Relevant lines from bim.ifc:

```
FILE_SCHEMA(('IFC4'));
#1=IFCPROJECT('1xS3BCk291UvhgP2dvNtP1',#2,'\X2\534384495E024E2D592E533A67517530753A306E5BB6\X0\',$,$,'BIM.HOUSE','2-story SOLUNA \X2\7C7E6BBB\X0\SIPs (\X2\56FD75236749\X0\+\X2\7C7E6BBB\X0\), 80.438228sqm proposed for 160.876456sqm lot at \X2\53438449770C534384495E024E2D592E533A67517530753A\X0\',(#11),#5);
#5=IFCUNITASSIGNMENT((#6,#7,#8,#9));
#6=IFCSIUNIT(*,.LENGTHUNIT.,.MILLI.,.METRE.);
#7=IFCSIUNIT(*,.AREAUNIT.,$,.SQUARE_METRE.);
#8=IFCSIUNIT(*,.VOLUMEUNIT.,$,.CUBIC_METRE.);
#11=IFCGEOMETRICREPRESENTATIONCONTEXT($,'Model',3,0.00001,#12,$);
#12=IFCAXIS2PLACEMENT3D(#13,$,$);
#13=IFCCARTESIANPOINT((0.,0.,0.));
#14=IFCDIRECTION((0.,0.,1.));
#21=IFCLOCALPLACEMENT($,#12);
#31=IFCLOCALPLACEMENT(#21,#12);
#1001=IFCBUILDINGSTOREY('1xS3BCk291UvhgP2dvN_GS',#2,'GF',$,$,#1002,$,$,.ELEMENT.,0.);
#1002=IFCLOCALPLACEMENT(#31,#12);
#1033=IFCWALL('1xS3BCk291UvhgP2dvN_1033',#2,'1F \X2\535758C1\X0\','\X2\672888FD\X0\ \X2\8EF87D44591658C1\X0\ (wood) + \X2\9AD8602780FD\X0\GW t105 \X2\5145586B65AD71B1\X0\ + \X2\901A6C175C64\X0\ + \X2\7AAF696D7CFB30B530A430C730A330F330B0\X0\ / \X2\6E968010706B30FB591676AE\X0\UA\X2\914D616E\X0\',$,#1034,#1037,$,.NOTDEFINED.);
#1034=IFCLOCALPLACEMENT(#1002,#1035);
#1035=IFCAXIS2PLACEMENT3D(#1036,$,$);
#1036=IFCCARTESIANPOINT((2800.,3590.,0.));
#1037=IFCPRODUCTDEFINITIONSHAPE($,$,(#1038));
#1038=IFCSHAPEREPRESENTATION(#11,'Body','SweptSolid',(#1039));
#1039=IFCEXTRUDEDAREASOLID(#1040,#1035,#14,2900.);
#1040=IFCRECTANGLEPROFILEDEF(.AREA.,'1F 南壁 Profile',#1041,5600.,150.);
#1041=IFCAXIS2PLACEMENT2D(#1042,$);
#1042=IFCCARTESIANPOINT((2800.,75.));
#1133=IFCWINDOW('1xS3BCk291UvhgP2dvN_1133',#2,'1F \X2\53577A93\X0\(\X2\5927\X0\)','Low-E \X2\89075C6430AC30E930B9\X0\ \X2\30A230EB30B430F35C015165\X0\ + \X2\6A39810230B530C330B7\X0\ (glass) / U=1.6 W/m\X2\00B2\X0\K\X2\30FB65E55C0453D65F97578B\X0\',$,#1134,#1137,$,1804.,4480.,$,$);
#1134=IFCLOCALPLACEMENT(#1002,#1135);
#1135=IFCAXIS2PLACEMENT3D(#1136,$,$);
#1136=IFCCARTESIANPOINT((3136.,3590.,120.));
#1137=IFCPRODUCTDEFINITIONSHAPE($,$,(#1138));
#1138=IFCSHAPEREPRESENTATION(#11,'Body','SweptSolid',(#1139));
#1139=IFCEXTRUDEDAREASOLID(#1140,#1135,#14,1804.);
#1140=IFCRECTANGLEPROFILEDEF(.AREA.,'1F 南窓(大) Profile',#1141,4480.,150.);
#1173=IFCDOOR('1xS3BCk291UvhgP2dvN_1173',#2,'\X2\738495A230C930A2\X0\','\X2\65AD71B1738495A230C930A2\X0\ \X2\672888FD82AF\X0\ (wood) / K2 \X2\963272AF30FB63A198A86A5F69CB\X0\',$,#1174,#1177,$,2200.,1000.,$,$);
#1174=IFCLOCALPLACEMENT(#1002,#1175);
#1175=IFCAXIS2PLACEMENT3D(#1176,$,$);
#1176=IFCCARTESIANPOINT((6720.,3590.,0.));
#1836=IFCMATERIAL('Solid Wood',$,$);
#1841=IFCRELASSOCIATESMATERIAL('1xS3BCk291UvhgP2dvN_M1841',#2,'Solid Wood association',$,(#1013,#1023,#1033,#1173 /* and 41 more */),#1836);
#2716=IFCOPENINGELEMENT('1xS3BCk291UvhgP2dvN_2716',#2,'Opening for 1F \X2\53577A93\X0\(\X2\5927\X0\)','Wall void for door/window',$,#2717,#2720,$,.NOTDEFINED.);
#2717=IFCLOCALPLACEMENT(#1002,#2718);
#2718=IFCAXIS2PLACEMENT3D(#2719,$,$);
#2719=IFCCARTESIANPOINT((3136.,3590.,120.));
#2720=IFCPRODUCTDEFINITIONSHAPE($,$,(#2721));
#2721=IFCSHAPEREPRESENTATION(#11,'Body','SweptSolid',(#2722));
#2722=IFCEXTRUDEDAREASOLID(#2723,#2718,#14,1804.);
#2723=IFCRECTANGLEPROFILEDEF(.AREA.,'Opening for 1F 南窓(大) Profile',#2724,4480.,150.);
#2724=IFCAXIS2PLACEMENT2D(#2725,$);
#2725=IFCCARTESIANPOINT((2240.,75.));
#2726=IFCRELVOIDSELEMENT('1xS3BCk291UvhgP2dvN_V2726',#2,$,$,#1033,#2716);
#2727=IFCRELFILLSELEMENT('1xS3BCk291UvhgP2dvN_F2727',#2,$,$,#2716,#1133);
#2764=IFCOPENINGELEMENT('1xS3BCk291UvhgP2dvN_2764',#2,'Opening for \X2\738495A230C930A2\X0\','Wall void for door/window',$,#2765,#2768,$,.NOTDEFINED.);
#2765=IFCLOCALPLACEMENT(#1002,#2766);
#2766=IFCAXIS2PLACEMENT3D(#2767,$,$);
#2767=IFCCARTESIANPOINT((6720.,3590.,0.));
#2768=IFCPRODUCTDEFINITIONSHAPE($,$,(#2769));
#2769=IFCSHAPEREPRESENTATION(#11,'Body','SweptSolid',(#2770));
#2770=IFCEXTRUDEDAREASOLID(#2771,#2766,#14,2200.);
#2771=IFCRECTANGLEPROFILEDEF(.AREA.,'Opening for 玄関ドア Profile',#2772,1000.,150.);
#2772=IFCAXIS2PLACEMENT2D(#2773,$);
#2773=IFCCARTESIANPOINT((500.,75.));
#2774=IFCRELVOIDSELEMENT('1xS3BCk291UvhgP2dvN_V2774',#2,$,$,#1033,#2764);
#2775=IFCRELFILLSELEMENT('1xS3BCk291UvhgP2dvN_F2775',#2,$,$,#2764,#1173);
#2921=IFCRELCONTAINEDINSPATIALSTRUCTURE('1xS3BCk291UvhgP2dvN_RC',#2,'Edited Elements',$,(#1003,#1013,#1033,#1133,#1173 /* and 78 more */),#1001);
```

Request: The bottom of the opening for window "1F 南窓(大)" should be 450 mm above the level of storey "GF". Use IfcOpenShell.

```python
import numpy as np
import ifcopenshell
import ifcopenshell.api.geometry
import ifcopenshell.geom
import ifcopenshell.util.element
import ifcopenshell.util.placement
import ifcopenshell.util.shape
import ifcopenshell.util.unit

model = ifcopenshell.open("bim.ifc")
unit_scale = ifcopenshell.util.unit.calculate_unit_scale(model)

window = model.by_id(1133)
opening = window.FillsVoids[0].RelatingOpeningElement
storey = ifcopenshell.util.element.get_container(window, ifc_class="IfcBuildingStorey")
level = ifcopenshell.util.placement.get_local_placement(storey.ObjectPlacement)[2, 3]

# The opening's origin need not be at the sill, so measure its lowest point.
shape = ifcopenshell.geom.create_shape(ifcopenshell.geom.settings(), opening)
bottom = ifcopenshell.util.shape.get_shape_bottom_elevation(shape, shape.geometry) / unit_scale
dz = level + 0.45 / unit_scale - bottom

shift = np.array([0.0, 0.0, dz])
# The window is not placed relative to its opening, so move both.
for product in (opening, window):
    matrix = ifcopenshell.util.placement.get_local_placement(product.ObjectPlacement)
    matrix[:3, 3] += shift
    ifcopenshell.api.geometry.edit_object_placement(model, product=product, matrix=matrix, is_si=False)

print(f"moved by {dz * unit_scale:+.3f} m")

model.write("bim_updated.ifc")
```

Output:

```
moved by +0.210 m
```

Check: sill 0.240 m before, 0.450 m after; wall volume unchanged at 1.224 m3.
